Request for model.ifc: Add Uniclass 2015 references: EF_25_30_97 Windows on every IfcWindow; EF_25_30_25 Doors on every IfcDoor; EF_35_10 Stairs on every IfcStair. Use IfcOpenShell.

First a look at what the model holds.

```python
import ifcopenshell

model = ifcopenshell.open("model.ifc")
print(model.schema)
print("classifications:", [c.Name for c in model.by_type("IfcClassification")])
for ifc_class in ("IfcDoor", "IfcRoof", "IfcStair", "IfcWall", "IfcWindow"):
    print(ifc_class, len(model.by_type(ifc_class)))
```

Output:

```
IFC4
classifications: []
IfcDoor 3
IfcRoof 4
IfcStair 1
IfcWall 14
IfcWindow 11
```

```python
import ifcopenshell
import ifcopenshell.api.classification

model = ifcopenshell.open("model.ifc")

system = ifcopenshell.api.classification.add_classification(model, classification="Uniclass 2015")

codes = {
    "IfcWindow": ("EF_25_30_97", "Windows"),
    "IfcDoor": ("EF_25_30_25", "Doors"),
    "IfcStair": ("EF_35_10", "Stairs"),
}
for ifc_class, (code, name) in codes.items():
    products = model.by_type(ifc_class)
    ifcopenshell.api.classification.add_reference(
        model, products=products, classification=system, identification=code, name=name
    )
    print(code, len(products))

model.write("model_rev.ifc")
```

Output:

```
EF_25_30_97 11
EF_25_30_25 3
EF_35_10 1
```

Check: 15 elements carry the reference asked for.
